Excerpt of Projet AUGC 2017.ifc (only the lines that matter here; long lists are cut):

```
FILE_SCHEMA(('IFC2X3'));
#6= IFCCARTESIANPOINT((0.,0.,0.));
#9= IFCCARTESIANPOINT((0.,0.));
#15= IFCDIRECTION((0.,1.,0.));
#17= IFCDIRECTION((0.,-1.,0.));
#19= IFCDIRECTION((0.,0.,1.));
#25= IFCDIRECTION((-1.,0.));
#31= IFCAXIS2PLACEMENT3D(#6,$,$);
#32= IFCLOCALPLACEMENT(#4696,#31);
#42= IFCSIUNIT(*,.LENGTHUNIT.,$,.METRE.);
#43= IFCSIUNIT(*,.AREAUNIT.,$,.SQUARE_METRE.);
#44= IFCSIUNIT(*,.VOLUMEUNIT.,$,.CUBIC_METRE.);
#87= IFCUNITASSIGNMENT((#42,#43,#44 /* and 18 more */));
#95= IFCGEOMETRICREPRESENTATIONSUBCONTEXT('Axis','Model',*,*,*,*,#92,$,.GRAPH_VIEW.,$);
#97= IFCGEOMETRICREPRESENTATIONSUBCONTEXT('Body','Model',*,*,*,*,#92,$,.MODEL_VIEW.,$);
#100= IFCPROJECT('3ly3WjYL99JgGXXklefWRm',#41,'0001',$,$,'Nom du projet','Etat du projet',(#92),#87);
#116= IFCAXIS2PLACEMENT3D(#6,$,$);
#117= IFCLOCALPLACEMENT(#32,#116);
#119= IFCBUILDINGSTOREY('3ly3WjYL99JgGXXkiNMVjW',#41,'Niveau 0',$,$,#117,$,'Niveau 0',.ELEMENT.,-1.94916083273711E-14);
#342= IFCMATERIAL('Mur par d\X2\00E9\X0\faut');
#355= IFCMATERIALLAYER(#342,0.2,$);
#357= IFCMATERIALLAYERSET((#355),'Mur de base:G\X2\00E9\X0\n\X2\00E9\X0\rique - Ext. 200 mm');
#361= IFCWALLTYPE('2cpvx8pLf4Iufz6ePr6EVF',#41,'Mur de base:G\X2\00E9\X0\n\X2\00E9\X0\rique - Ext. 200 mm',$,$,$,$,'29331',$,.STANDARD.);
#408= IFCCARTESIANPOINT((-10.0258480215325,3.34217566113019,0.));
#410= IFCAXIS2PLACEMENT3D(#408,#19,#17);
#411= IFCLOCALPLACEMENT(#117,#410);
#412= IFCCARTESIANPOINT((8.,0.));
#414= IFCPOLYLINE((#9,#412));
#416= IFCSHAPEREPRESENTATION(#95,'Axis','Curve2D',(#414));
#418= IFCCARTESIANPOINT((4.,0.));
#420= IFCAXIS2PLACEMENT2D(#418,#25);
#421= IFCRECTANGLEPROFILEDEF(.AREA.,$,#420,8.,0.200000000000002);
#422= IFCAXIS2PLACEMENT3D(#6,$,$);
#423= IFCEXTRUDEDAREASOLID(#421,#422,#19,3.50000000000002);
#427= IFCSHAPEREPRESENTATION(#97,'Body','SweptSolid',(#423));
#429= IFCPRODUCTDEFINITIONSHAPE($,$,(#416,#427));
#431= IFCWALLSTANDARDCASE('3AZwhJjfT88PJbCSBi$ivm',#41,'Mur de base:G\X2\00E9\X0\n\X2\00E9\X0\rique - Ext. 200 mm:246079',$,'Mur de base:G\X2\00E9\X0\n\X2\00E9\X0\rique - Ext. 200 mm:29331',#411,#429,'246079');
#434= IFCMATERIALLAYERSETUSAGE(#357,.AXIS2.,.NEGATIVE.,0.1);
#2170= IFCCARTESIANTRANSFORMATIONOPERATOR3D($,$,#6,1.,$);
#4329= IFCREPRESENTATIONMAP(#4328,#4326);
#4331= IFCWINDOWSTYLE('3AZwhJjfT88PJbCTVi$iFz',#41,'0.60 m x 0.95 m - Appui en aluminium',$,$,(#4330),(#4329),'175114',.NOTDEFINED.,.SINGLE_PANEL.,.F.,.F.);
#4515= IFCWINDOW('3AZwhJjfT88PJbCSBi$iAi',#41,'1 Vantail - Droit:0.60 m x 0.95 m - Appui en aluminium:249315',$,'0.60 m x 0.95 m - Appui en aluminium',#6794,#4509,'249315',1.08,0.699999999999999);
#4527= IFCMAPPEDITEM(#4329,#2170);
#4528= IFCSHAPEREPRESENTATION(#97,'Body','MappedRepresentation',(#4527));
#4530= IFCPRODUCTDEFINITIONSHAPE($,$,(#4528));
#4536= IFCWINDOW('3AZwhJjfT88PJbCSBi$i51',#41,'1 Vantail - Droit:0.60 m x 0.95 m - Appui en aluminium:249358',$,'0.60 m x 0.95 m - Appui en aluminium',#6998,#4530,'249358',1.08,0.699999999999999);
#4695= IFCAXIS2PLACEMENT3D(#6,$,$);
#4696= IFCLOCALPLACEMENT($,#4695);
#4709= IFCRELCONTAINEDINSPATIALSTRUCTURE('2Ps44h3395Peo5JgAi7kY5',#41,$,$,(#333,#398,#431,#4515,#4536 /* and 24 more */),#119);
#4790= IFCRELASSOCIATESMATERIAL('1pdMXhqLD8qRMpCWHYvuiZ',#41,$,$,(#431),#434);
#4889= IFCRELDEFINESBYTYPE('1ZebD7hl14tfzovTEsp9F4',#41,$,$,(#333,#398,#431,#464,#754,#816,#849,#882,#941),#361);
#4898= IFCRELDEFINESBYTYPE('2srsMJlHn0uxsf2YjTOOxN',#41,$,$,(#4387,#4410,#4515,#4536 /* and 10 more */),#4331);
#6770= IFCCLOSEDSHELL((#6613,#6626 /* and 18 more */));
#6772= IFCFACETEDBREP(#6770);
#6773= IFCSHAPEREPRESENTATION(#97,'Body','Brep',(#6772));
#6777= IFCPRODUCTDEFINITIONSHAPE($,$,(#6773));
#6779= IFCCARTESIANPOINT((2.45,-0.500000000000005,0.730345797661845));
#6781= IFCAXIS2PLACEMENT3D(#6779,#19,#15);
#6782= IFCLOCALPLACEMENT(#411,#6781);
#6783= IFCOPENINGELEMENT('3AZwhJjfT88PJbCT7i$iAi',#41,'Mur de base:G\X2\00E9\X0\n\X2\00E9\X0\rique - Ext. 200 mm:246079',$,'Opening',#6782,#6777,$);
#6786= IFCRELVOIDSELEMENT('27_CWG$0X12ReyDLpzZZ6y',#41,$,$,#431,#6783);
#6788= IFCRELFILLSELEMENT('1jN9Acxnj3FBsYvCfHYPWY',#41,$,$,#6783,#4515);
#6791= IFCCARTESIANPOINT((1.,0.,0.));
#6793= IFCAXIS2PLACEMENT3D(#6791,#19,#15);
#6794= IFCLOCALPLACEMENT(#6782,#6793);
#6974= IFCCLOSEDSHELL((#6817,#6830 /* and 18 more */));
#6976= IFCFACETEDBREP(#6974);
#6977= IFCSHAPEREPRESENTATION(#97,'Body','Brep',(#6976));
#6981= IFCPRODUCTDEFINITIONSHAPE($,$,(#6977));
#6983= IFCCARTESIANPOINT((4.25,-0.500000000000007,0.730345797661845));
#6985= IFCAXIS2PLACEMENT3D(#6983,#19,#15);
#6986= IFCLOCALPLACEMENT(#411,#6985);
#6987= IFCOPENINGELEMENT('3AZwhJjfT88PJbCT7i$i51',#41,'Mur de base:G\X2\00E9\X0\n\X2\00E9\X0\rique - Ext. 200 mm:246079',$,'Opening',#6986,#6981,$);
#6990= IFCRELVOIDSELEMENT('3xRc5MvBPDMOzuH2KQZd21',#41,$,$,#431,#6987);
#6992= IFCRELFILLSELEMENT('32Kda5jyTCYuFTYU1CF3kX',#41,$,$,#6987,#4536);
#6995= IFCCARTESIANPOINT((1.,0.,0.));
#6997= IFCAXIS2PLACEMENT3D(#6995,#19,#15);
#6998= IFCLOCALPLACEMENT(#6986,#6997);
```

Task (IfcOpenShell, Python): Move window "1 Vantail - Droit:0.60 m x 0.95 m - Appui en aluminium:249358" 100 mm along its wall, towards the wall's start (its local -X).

```python
import ifcopenshell
import ifcopenshell.api.geometry
import ifcopenshell.util.placement
import ifcopenshell.util.unit

model = ifcopenshell.open("Projet AUGC 2017.ifc")
unit_scale = ifcopenshell.util.unit.calculate_unit_scale(model)

window = model.by_guid("3AZwhJjfT88PJbCSBi$i51")
opening = window.FillsVoids[0].RelatingOpeningElement
wall = opening.VoidsElements[0].RelatingBuildingElement

wall_matrix = ifcopenshell.util.placement.get_local_placement(wall.ObjectPlacement)
shift = wall_matrix[:3, 0] * -0.1 / unit_scale
before = ifcopenshell.util.placement.get_local_placement(window.ObjectPlacement)[:3, 3].copy()

# The window is placed relative to its opening, so it follows when the opening moves.
matrix = ifcopenshell.util.placement.get_local_placement(opening.ObjectPlacement)
matrix[:3, 3] += shift
ifcopenshell.api.geometry.edit_object_placement(
    model, product=opening, matrix=matrix, is_si=False, should_transform_children=True
)

after = ifcopenshell.util.placement.get_local_placement(window.ObjectPlacement)[:3, 3]
print("window moved by", (after - before).round(3) + 0.0)

model.write("Projet AUGC 2017_rev.ifc")
```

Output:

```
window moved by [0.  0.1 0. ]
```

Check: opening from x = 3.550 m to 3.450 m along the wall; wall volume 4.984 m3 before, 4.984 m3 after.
